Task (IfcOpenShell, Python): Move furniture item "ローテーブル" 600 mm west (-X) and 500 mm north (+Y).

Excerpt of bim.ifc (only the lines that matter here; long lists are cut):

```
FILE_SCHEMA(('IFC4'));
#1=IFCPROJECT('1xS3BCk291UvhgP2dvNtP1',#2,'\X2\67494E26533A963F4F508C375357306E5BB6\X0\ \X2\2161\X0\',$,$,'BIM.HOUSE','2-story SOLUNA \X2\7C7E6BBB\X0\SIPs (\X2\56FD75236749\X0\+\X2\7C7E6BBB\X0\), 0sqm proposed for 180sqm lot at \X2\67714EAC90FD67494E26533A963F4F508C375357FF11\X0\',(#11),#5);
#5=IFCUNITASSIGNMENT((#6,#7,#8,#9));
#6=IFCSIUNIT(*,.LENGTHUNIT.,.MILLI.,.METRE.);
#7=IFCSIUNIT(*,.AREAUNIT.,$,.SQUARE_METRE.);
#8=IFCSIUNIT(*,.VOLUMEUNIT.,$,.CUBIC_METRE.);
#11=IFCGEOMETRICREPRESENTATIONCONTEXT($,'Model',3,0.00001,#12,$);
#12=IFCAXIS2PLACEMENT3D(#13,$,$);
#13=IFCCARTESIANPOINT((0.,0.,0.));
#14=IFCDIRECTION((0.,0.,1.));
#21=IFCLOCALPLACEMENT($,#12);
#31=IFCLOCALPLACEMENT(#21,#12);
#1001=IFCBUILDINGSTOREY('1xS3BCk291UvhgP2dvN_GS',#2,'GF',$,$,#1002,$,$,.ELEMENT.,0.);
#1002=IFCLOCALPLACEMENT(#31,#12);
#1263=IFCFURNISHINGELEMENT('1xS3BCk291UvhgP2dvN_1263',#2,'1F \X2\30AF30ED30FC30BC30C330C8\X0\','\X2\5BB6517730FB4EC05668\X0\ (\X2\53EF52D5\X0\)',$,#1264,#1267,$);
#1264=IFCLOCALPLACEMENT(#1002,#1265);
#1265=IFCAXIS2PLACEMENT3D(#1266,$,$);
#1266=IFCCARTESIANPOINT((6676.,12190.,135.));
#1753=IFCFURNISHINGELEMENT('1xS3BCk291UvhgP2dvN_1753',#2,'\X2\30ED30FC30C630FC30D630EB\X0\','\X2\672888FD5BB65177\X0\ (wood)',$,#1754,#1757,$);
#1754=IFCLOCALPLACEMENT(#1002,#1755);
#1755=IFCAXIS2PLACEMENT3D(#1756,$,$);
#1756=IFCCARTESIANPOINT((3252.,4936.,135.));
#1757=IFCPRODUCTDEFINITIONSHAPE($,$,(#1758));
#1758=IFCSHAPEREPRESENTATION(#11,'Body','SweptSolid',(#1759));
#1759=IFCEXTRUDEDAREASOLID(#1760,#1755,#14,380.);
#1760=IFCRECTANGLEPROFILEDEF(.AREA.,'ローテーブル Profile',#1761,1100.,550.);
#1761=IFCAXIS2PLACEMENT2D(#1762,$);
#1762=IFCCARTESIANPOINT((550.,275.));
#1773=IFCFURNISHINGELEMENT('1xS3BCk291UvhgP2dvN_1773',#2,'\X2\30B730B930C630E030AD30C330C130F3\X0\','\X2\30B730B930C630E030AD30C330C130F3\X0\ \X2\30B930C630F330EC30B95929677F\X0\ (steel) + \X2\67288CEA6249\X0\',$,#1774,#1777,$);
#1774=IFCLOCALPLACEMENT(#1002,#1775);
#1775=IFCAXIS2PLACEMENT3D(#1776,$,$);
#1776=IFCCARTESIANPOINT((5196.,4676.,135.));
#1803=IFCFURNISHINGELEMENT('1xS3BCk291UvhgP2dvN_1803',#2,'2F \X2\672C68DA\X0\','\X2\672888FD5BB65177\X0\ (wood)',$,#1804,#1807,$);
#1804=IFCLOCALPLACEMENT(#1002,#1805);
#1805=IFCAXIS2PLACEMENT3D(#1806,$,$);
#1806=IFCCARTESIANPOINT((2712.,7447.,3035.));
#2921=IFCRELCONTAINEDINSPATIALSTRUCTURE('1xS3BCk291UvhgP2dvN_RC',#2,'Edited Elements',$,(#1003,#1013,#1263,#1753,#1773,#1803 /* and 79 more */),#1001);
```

```python
import ifcopenshell
import ifcopenshell.api.geometry
import ifcopenshell.util.placement
import ifcopenshell.util.unit

model = ifcopenshell.open("bim.ifc")
unit_scale = ifcopenshell.util.unit.calculate_unit_scale(model)

item = model.by_id(1753)
matrix = ifcopenshell.util.placement.get_local_placement(item.ObjectPlacement)
matrix[0, 3] -= 0.6 / unit_scale
matrix[1, 3] += 0.5 / unit_scale
ifcopenshell.api.geometry.edit_object_placement(model, product=item, matrix=matrix, is_si=False)

print(ifcopenshell.util.placement.get_local_placement(item.ObjectPlacement).round(3) + 0.0)

model.write("bim_rev.ifc")
```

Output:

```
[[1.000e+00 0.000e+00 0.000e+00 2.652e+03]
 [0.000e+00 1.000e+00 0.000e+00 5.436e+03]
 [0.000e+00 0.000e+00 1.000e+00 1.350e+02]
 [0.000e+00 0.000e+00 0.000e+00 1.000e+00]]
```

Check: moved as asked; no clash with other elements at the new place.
